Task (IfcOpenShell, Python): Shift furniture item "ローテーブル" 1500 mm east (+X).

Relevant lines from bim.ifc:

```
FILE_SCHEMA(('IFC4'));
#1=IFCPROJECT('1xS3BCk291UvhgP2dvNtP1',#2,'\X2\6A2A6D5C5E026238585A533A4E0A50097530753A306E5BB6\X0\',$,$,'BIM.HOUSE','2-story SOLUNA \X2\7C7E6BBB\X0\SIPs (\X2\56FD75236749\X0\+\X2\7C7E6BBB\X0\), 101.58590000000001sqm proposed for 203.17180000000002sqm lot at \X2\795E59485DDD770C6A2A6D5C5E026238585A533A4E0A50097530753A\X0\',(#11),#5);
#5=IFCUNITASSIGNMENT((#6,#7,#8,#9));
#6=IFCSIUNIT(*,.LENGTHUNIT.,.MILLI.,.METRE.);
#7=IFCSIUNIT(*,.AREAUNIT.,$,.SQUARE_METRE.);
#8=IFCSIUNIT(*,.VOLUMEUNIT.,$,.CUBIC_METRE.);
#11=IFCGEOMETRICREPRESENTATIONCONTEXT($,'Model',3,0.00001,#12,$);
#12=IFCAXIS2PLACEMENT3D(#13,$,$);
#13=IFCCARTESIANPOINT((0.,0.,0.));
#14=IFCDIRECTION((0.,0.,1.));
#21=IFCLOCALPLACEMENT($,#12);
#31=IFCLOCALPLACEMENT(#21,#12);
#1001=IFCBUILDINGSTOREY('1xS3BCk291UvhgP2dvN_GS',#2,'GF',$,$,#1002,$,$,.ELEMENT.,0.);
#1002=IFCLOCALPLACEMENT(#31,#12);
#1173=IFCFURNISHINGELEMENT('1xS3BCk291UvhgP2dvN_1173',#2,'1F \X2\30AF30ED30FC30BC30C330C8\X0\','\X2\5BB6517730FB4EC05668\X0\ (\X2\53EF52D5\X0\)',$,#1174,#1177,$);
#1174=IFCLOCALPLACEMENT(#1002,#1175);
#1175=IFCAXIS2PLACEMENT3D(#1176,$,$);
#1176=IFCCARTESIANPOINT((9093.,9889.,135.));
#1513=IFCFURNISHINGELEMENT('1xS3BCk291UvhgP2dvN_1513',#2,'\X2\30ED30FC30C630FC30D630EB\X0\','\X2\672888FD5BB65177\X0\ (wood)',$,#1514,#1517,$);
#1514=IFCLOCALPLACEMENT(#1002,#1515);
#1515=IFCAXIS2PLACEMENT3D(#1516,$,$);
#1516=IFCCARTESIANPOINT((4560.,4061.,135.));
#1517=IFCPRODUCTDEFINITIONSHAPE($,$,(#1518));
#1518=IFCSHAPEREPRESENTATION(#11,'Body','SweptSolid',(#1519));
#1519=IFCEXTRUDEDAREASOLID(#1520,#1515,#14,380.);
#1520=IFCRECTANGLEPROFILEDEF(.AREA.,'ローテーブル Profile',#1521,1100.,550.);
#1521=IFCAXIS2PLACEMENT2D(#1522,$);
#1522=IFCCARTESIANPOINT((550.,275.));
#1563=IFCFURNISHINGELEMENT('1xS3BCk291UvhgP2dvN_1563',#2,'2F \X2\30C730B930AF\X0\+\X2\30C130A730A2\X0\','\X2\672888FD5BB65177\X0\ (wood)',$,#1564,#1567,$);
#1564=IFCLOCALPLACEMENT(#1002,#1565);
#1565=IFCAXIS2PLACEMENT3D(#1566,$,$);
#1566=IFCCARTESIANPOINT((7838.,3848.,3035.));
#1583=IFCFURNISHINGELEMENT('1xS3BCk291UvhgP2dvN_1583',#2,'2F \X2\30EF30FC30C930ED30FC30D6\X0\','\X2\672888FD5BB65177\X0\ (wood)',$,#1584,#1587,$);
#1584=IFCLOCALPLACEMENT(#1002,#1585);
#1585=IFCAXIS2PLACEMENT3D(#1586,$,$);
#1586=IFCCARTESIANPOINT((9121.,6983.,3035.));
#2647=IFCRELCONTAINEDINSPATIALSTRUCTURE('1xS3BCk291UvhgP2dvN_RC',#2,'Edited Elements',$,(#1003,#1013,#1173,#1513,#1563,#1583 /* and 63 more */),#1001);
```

```python
import ifcopenshell
import ifcopenshell.api.geometry
import ifcopenshell.util.placement
import ifcopenshell.util.unit

model = ifcopenshell.open("bim.ifc")
unit_scale = ifcopenshell.util.unit.calculate_unit_scale(model)

item = model.by_guid("1xS3BCk291UvhgP2dvN_1513")
matrix = ifcopenshell.util.placement.get_local_placement(item.ObjectPlacement)
matrix[0, 3] += 1.5 / unit_scale
ifcopenshell.api.geometry.edit_object_placement(model, product=item, matrix=matrix, is_si=False)

print(ifcopenshell.util.placement.get_local_placement(item.ObjectPlacement).round(3) + 0.0)

model.write("bim_edited.ifc")
```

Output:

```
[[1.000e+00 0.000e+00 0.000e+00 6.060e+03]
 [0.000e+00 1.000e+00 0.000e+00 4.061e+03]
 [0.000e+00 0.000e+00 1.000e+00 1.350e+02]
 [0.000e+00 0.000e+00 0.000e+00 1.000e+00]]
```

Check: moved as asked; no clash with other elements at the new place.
